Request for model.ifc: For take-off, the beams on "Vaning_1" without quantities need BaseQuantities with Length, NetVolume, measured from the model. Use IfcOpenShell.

First a look at what the model holds.

```python
import ifcopenshell
import ifcopenshell.util.element
import ifcopenshell.util.unit

model = ifcopenshell.open("model.ifc")
print(model.schema)
for unit_type in ("LENGTHUNIT", "AREAUNIT", "VOLUMEUNIT"):
    print(unit_type, ifcopenshell.util.unit.calculate_unit_scale(model, unit_type))
storey = next(s for s in model.by_type("IfcBuildingStorey") if s.Name == "Vaning_1")
beams = [e for e in ifcopenshell.util.element.get_decomposition(storey) if e.is_a("IfcBeam")]
for e in sorted(beams, key=lambda e: e.id()):
    print(e.id(), e.is_a(), e.Name, list(ifcopenshell.util.element.get_psets(e, qtos_only=True)), sep=" | ")
```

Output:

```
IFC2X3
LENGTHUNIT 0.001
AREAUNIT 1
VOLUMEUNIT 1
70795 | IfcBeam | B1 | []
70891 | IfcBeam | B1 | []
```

```python
import ifcopenshell
import ifcopenshell.api.pset
import ifcopenshell.geom
import ifcopenshell.util.element
import ifcopenshell.util.shape
import ifcopenshell.util.unit

model = ifcopenshell.open("model.ifc")
unit_scale = ifcopenshell.util.unit.calculate_unit_scale(model)
volume_scale = ifcopenshell.util.unit.calculate_unit_scale(model, "VOLUMEUNIT")
settings = ifcopenshell.geom.settings()

storey = next(s for s in model.by_type("IfcBuildingStorey") if s.Name == "Vaning_1")
beams = [e for e in ifcopenshell.util.element.get_decomposition(storey) if e.is_a("IfcBeam")]

for e in sorted(beams, key=lambda e: e.id()):
    if ifcopenshell.util.element.get_psets(e, qtos_only=True, should_inherit=False):
        continue
    # Geometry comes back in metres, in the element's own axes.
    shape = ifcopenshell.geom.create_shape(settings, e)
    values = {
        "Length": ifcopenshell.util.shape.get_max_xyz(shape.geometry) / unit_scale,
        "NetVolume": ifcopenshell.util.shape.get_volume(shape.geometry) / volume_scale,
    }
    qto = ifcopenshell.api.pset.add_qto(model, product=e, name="BaseQuantities")
    ifcopenshell.api.pset.edit_qto(model, qto=qto, properties=values)
    print(e.id(), {k: round(v, 3) for k, v in values.items()})

model.write("model-out.ifc")
```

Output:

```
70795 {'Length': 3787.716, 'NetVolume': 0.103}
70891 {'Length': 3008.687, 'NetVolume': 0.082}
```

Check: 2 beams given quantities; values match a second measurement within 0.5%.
